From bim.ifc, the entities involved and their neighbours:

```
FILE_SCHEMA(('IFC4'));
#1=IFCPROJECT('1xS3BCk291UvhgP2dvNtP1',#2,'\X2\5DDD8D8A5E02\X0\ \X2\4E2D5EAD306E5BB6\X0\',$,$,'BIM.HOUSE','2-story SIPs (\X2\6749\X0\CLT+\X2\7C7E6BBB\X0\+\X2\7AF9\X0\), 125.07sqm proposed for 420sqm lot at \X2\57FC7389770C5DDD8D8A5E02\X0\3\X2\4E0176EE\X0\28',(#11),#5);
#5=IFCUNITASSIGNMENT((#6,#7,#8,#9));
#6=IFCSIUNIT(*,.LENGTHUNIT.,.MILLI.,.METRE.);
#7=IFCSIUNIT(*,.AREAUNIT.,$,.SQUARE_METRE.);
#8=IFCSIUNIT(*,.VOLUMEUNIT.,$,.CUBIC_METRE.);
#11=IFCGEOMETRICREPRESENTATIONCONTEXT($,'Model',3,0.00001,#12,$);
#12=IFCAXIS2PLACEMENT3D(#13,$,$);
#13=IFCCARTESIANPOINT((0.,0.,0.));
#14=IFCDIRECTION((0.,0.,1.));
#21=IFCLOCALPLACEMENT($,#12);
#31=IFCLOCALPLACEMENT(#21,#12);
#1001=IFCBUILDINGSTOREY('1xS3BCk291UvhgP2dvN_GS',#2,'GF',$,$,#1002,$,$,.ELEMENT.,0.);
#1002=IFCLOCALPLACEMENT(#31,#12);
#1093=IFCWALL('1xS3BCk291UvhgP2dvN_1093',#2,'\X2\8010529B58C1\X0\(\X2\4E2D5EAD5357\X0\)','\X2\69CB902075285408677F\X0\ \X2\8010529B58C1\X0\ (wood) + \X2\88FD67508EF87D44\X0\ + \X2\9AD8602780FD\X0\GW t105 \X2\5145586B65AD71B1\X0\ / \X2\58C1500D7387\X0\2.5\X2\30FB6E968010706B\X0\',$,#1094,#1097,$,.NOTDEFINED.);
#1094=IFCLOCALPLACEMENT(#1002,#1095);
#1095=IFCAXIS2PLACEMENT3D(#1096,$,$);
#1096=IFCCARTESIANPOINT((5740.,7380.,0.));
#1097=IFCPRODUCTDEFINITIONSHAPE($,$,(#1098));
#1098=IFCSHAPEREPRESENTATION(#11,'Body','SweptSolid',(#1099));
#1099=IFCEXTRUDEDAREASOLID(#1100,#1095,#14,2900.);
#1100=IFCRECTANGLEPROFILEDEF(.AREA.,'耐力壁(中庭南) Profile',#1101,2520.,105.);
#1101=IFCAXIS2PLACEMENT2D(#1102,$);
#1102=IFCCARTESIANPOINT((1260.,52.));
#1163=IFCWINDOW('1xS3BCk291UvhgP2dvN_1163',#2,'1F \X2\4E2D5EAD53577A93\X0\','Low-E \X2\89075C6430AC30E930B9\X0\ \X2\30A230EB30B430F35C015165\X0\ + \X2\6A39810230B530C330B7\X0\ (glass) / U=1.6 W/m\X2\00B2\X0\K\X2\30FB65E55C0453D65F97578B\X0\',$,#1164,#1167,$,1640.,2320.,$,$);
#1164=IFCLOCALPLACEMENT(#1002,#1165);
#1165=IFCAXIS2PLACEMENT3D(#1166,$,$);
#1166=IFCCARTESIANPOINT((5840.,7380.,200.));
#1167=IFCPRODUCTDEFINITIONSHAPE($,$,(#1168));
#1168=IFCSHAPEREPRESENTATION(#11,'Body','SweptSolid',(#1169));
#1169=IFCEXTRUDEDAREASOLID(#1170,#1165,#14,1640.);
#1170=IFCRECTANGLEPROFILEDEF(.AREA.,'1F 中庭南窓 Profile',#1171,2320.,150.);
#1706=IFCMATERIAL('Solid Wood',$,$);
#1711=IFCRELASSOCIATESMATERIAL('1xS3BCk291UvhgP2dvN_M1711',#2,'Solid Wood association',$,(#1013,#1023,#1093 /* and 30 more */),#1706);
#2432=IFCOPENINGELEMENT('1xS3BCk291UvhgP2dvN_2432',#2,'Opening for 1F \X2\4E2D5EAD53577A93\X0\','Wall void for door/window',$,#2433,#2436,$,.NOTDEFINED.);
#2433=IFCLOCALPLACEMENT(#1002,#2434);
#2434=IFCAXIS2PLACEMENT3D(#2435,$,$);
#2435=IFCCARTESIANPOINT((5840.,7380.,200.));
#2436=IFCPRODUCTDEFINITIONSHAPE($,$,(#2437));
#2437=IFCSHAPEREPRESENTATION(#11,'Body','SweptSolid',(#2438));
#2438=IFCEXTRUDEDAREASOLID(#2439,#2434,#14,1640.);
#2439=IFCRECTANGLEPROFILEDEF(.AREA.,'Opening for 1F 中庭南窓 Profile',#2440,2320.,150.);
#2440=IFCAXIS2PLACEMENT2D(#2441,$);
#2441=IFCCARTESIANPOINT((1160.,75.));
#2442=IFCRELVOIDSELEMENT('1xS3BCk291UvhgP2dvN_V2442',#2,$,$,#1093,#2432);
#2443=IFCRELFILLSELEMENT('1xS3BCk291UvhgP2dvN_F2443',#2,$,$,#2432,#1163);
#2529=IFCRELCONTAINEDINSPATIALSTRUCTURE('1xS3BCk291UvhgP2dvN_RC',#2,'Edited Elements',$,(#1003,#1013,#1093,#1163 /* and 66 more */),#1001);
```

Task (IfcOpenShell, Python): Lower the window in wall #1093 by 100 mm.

```python
import numpy as np
import ifcopenshell
import ifcopenshell.api.geometry
import ifcopenshell.util.placement
import ifcopenshell.util.unit

model = ifcopenshell.open("bim.ifc")
unit_scale = ifcopenshell.util.unit.calculate_unit_scale(model)

window = model.by_guid("1xS3BCk291UvhgP2dvN_1163")
opening = window.FillsVoids[0].RelatingOpeningElement
dz = -100.0

shift = np.array([0.0, 0.0, dz])
# The window is not placed relative to its opening, so move both.
for product in (opening, window):
    matrix = ifcopenshell.util.placement.get_local_placement(product.ObjectPlacement)
    matrix[:3, 3] += shift
    ifcopenshell.api.geometry.edit_object_placement(model, product=product, matrix=matrix, is_si=False)

print(f"moved by {dz * unit_scale:+.3f} m")

model.write("bim_v2.ifc")
```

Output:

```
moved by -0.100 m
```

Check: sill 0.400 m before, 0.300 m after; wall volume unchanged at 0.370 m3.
